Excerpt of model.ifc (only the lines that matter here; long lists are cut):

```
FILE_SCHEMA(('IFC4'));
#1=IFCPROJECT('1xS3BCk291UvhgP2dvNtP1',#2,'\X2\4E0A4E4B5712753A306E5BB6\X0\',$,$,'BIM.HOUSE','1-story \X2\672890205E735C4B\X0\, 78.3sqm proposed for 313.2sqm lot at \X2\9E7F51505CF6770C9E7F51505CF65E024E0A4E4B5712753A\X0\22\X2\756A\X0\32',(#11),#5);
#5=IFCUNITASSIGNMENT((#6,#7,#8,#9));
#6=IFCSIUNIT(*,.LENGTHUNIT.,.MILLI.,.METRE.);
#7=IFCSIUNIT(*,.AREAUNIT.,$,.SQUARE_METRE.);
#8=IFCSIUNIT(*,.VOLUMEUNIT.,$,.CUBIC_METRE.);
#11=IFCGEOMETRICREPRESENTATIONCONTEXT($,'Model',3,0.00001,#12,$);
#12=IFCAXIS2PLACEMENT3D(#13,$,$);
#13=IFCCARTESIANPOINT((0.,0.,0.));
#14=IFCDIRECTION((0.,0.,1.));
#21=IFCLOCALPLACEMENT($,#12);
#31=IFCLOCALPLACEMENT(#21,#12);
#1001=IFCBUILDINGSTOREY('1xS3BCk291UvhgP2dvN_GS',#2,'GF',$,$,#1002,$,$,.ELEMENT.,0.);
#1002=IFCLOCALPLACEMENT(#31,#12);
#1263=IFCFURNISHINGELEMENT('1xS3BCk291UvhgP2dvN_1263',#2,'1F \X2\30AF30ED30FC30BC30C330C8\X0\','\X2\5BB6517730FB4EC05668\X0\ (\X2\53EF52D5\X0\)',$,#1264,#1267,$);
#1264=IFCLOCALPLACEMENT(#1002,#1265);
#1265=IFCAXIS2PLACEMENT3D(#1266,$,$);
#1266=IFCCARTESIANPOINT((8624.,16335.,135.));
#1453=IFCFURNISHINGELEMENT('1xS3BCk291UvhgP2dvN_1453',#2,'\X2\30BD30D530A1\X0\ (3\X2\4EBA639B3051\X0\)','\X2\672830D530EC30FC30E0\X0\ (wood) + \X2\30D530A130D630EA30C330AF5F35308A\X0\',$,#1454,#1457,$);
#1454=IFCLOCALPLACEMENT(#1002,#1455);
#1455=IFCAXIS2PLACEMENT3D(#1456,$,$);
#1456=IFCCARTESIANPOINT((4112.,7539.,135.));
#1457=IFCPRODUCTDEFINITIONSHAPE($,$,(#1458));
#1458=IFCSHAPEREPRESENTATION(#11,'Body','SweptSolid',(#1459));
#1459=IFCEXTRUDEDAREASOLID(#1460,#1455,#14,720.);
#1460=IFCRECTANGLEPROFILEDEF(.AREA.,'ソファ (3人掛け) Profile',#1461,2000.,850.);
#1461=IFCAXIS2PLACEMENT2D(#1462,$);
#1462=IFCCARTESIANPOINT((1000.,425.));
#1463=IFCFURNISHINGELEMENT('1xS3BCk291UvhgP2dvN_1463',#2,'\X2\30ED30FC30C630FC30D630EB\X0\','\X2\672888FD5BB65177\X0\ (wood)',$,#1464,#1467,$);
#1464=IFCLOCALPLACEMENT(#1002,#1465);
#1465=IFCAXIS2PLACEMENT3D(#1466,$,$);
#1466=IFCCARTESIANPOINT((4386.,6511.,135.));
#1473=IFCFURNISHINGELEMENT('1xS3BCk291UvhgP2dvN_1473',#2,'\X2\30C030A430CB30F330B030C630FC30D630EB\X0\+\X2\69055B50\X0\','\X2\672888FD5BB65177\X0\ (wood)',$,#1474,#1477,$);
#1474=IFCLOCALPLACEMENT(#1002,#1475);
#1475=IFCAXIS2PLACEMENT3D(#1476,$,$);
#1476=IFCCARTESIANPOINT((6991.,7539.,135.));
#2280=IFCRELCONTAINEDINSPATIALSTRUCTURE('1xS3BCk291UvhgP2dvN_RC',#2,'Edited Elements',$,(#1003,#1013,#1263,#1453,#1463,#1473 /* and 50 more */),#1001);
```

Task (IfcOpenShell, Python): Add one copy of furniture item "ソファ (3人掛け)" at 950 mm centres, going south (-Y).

```python
import numpy as np
import ifcopenshell
import ifcopenshell.api.geometry
import ifcopenshell.api.root
import ifcopenshell.util.element
import ifcopenshell.util.placement
import ifcopenshell.util.unit

model = ifcopenshell.open("model.ifc")
unit_scale = ifcopenshell.util.unit.calculate_unit_scale(model)


def reuse_history(source, copy):
    """copy_class also copies each property set's owner history, people and application; keep the originals."""
    for rel in copy.IsDefinedBy:
        if rel.is_a("IfcRelDefinesByProperties") and (history := rel.RelatingPropertyDefinition.OwnerHistory):
            rel.RelatingPropertyDefinition.OwnerHistory = source.OwnerHistory
            ifcopenshell.util.element.remove_deep2(model, history)


source = model.by_id(1453)
base = ifcopenshell.util.placement.get_local_placement(source.ObjectPlacement)
step = np.array([0.0, -1.0, 0.0]) * 0.95 / unit_scale

for i in range(1, 2):
    copy = ifcopenshell.api.root.copy_class(model, product=source)
    copy.Representation = ifcopenshell.util.element.copy_deep(
        model, source.Representation, exclude=["IfcGeometricRepresentationContext", "IfcRepresentationMap"]
    )
    reuse_history(source, copy)
    matrix = base.copy()
    matrix[:3, 3] += i * step
    print("added at", matrix[:3, 3].round(3) + 0.0)
    ifcopenshell.api.geometry.edit_object_placement(model, product=copy, matrix=matrix, is_si=False)

model.write("model_edited.ifc")
```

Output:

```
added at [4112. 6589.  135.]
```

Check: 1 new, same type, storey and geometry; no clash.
